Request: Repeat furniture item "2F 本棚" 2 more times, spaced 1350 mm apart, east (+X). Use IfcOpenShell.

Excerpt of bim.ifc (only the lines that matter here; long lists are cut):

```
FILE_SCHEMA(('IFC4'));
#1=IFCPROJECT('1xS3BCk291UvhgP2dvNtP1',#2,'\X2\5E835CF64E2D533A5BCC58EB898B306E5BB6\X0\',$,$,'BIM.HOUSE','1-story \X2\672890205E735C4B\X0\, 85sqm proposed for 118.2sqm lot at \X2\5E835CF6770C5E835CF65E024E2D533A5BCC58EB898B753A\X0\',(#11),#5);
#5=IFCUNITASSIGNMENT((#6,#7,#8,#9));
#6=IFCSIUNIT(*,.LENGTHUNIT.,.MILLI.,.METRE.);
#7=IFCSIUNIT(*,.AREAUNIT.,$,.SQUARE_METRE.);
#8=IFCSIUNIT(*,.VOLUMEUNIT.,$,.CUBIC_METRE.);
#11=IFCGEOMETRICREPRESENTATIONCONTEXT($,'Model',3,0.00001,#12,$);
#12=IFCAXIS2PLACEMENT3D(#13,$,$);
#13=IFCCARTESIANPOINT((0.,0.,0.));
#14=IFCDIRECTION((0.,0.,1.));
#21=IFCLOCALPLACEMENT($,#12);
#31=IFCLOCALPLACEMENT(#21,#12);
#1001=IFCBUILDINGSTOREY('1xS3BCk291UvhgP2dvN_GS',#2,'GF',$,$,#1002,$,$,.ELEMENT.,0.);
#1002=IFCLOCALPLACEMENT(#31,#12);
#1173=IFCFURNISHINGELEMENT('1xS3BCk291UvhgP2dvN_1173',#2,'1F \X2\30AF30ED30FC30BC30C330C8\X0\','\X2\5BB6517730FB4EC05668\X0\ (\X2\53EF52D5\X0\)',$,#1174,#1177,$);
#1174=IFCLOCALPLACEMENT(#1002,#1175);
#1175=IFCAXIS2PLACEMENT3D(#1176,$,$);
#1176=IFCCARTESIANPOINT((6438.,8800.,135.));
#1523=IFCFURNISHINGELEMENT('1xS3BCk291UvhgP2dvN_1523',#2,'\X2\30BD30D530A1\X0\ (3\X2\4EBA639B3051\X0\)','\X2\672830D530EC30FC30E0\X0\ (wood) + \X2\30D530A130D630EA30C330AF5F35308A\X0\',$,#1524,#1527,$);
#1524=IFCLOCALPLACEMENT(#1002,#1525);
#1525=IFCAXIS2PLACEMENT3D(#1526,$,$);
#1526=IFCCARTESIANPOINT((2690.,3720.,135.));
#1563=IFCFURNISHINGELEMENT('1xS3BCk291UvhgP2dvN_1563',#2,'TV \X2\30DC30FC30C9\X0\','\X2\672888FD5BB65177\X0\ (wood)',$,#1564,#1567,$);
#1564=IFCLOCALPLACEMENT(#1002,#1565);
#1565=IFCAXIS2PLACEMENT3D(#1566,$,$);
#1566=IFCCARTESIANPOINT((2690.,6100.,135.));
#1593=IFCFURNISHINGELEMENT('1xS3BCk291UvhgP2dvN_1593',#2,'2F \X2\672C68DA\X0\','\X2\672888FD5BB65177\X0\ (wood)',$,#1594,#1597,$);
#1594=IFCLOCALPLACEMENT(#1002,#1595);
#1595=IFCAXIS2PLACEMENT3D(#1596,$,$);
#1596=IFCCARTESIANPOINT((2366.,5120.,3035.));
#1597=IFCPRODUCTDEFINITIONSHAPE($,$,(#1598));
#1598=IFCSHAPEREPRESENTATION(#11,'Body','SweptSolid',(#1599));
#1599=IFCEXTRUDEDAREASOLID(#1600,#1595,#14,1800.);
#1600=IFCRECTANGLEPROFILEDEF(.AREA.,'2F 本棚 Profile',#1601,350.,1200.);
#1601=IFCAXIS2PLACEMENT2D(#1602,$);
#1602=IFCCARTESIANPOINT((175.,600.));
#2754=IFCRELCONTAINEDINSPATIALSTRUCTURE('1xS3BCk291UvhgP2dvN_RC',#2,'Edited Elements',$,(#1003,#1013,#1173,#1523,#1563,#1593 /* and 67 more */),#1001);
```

```python
import numpy as np
import ifcopenshell
import ifcopenshell.api.geometry
import ifcopenshell.api.root
import ifcopenshell.util.element
import ifcopenshell.util.placement
import ifcopenshell.util.unit

model = ifcopenshell.open("bim.ifc")
unit_scale = ifcopenshell.util.unit.calculate_unit_scale(model)


def reuse_history(source, copy):
    """copy_class also copies each property set's owner history, people and application; keep the originals."""
    for rel in copy.IsDefinedBy:
        if rel.is_a("IfcRelDefinesByProperties") and (history := rel.RelatingPropertyDefinition.OwnerHistory):
            rel.RelatingPropertyDefinition.OwnerHistory = source.OwnerHistory
            ifcopenshell.util.element.remove_deep2(model, history)


source = model.by_guid("1xS3BCk291UvhgP2dvN_1593")
base = ifcopenshell.util.placement.get_local_placement(source.ObjectPlacement)
step = np.array([1.0, 0.0, 0.0]) * 1.35 / unit_scale

for i in range(1, 3):
    copy = ifcopenshell.api.root.copy_class(model, product=source)
    copy.Representation = ifcopenshell.util.element.copy_deep(
        model, source.Representation, exclude=["IfcGeometricRepresentationContext", "IfcRepresentationMap"]
    )
    reuse_history(source, copy)
    matrix = base.copy()
    matrix[:3, 3] += i * step
    print("added at", matrix[:3, 3].round(3) + 0.0)
    ifcopenshell.api.geometry.edit_object_placement(model, product=copy, matrix=matrix, is_si=False)

model.write("bim-out.ifc")
```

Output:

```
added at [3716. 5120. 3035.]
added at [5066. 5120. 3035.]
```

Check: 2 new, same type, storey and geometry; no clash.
